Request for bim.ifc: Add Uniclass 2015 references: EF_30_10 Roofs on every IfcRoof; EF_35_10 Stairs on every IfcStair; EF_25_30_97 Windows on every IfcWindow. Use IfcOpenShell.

First a look at what the model holds.

```python
import ifcopenshell

model = ifcopenshell.open("bim.ifc")
print(model.schema)
print("classifications:", [c.Name for c in model.by_type("IfcClassification")])
for ifc_class in ("IfcDoor", "IfcRoof", "IfcStair", "IfcWall", "IfcWindow"):
    print(ifc_class, len(model.by_type(ifc_class)))
```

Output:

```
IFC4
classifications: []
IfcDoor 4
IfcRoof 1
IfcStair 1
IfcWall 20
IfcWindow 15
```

```python
import ifcopenshell
import ifcopenshell.api.classification

model = ifcopenshell.open("bim.ifc")

system = ifcopenshell.api.classification.add_classification(model, classification="Uniclass 2015")

codes = {
    "IfcRoof": ("EF_30_10", "Roofs"),
    "IfcStair": ("EF_35_10", "Stairs"),
    "IfcWindow": ("EF_25_30_97", "Windows"),
}
for ifc_class, (code, name) in codes.items():
    products = model.by_type(ifc_class)
    ifcopenshell.api.classification.add_reference(
        model, products=products, classification=system, identification=code, name=name
    )
    print(code, len(products))

model.write("bim_rev.ifc")
```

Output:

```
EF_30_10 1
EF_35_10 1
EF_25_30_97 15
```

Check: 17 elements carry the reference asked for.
